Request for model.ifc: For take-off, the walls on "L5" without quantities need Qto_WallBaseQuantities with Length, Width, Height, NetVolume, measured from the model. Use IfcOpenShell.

First a look at what the model holds.

```python
import ifcopenshell
import ifcopenshell.util.element
import ifcopenshell.util.unit

model = ifcopenshell.open("model.ifc")
print(model.schema)
for unit_type in ("LENGTHUNIT", "AREAUNIT", "VOLUMEUNIT"):
    print(unit_type, ifcopenshell.util.unit.calculate_unit_scale(model, unit_type))
storey = next(s for s in model.by_type("IfcBuildingStorey") if s.Name == "L5")
walls = [e for e in ifcopenshell.util.element.get_decomposition(storey) if e.is_a("IfcWall")]
for e in sorted(walls, key=lambda e: e.id()):
    print(e.id(), e.is_a(), e.Name, list(ifcopenshell.util.element.get_psets(e, qtos_only=True)), sep=" | ")
```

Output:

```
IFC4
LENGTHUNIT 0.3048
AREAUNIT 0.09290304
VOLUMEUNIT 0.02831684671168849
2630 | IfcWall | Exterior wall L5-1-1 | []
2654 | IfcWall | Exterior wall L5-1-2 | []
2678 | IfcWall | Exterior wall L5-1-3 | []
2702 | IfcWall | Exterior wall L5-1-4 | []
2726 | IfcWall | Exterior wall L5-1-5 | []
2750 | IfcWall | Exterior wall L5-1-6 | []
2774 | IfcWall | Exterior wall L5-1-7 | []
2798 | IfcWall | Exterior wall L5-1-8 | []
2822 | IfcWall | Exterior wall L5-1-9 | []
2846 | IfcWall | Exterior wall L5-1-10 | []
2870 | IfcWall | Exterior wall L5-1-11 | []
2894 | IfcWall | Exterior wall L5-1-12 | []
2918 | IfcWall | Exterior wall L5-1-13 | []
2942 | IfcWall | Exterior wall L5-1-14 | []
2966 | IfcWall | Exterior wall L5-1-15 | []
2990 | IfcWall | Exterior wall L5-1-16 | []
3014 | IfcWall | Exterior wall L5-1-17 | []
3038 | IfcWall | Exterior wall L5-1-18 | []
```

```python
import ifcopenshell
import ifcopenshell.api.pset
import ifcopenshell.geom
import ifcopenshell.util.element
import ifcopenshell.util.shape
import ifcopenshell.util.unit

model = ifcopenshell.open("model.ifc")
unit_scale = ifcopenshell.util.unit.calculate_unit_scale(model)
volume_scale = ifcopenshell.util.unit.calculate_unit_scale(model, "VOLUMEUNIT")
settings = ifcopenshell.geom.settings()

storey = next(s for s in model.by_type("IfcBuildingStorey") if s.Name == "L5")
walls = [e for e in ifcopenshell.util.element.get_decomposition(storey) if e.is_a("IfcWall")]

for e in sorted(walls, key=lambda e: e.id()):
    if ifcopenshell.util.element.get_psets(e, qtos_only=True, should_inherit=False):
        continue
    # Geometry comes back in metres, in the element's own axes.
    shape = ifcopenshell.geom.create_shape(settings, e)
    values = {
        "Length": ifcopenshell.util.shape.get_x(shape.geometry) / unit_scale,
        "Width": ifcopenshell.util.shape.get_y(shape.geometry) / unit_scale,
        "Height": ifcopenshell.util.shape.get_z(shape.geometry) / unit_scale,
        "NetVolume": ifcopenshell.util.shape.get_volume(shape.geometry) / volume_scale,
    }
    qto = ifcopenshell.api.pset.add_qto(model, product=e, name="Qto_WallBaseQuantities")
    ifcopenshell.api.pset.edit_qto(model, qto=qto, properties=values)
    print(e.id(), {k: round(v, 3) for k, v in values.items()})

model.write("model_v2.ifc")
```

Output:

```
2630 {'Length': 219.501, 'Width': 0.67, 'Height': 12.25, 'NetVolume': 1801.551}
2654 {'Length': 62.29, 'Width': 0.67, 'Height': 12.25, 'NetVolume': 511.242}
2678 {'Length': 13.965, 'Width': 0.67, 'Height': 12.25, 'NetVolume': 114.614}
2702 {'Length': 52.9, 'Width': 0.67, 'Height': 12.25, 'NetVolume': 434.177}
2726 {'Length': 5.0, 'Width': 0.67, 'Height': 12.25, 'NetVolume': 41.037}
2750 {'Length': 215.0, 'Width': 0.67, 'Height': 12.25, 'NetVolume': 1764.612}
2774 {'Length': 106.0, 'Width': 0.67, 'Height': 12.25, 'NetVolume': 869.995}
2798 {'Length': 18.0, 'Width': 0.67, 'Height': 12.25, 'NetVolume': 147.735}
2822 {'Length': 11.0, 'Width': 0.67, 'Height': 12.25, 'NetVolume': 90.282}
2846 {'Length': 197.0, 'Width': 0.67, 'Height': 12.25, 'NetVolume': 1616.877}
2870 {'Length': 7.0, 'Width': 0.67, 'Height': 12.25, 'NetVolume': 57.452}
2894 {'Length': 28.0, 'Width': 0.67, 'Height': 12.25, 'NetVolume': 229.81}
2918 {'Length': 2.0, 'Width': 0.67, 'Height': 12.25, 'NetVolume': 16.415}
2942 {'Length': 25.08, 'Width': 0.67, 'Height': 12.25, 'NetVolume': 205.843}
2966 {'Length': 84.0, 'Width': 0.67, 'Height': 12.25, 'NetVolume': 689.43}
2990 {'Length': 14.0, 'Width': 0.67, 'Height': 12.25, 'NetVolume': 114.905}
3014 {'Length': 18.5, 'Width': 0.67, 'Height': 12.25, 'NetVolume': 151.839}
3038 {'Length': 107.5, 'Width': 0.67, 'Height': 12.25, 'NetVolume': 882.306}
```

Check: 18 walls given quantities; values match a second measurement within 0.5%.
